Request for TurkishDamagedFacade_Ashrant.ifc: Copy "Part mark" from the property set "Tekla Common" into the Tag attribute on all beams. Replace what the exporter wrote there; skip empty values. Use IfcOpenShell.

First a look at what the model holds.

```python
import ifcopenshell
import ifcopenshell.util.element

model = ifcopenshell.open("TurkishDamagedFacade_Ashrant.ifc")
print(model.schema)
beams = model.by_type("IfcBeam")
print(len(beams), "beams")
for e in beams[:8]:
    source = ifcopenshell.util.element.get_pset(e, "Tekla Common", "Part mark")
    target = e.Tag
    print(e.id(), repr(source), repr(target), sep=" | ")
```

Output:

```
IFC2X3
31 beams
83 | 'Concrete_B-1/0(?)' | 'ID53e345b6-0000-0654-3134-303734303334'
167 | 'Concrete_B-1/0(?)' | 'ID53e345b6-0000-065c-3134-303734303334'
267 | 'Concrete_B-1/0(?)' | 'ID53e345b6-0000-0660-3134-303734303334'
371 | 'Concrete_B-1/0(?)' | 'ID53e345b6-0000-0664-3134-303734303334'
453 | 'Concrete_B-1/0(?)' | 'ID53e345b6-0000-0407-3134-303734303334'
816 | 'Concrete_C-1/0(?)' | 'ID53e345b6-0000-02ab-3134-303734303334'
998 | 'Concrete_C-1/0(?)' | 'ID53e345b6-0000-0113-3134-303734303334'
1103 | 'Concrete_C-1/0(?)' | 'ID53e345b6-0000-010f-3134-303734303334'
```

```python
import ifcopenshell
import ifcopenshell.util.element

model = ifcopenshell.open("TurkishDamagedFacade_Ashrant.ifc")

count = 0
for e in model.by_type("IfcBeam"):
    value = ifcopenshell.util.element.get_pset(e, "Tekla Common", "Part mark")
    current = e.Tag
    if not value or not value.strip() or current == value:
        continue
    e.Tag = value
    count += 1

print(count, "beams updated")

model.write("TurkishDamagedFacade_Ashrant_v2.ifc")
```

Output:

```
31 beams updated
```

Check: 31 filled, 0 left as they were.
